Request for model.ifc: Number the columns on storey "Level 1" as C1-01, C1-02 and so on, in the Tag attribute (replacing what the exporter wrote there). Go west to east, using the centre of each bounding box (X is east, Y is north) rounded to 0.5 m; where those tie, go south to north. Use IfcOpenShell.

First a look at what the model holds.

```python
import ifcopenshell
import ifcopenshell.util.element
import ifcopenshell.util.placement

model = ifcopenshell.open("model.ifc")
print(model.schema)
storey = next(s for s in model.by_type("IfcBuildingStorey") if s.Name == "Level 1")
columns = [e for e in ifcopenshell.util.element.get_decomposition(storey) if e.is_a("IfcColumn")]
for e in sorted(columns, key=lambda e: e.id()):
    origin = ifcopenshell.util.placement.get_local_placement(e.ObjectPlacement)[:3, 3]
    print(e.id(), e.Tag, e.Name, origin.round(2) + 0.0, sep=" | ")
```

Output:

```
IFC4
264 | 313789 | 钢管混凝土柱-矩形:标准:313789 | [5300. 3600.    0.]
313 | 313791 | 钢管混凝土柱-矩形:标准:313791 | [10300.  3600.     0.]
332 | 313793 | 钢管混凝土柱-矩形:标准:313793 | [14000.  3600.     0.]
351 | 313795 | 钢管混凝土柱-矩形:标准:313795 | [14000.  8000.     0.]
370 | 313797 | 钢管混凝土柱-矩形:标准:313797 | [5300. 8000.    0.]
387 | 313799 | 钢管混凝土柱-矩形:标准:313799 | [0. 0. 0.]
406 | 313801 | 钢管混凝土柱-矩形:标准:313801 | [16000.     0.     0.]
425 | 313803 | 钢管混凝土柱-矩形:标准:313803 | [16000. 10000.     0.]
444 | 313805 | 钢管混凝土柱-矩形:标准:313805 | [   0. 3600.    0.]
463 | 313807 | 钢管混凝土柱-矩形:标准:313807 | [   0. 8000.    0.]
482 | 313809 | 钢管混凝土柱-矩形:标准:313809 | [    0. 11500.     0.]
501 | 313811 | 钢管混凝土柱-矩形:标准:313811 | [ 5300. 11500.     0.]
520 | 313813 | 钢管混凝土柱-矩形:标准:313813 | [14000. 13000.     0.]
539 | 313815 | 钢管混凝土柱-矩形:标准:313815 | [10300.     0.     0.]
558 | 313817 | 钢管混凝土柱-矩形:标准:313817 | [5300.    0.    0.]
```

```python
import ifcopenshell
import ifcopenshell.geom
import ifcopenshell.util.element
import ifcopenshell.util.shape

model = ifcopenshell.open("model.ifc")
settings = ifcopenshell.geom.settings()
settings.set("use-world-coords", True)


def centre(element):
    shape = ifcopenshell.geom.create_shape(settings, element)
    return ifcopenshell.util.shape.get_bbox_centroid(shape.geometry)


storey = next(s for s in model.by_type("IfcBuildingStorey") if s.Name == "Level 1")
columns = [e for e in ifcopenshell.util.element.get_decomposition(storey) if e.is_a("IfcColumn")]

# Insertion points can sit at a corner or the storey origin, so sort by the geometry (in metres).
centres = {e: centre(e) for e in columns}
columns.sort(key=lambda e: (round(centres[e][0] / 0.5), centres[e][1]))

for i, e in enumerate(columns, start=1):
    number = f"C1-{i:02d}"
    e.Tag = number
    print(e.id(), number)

model.write("model_updated.ifc")
```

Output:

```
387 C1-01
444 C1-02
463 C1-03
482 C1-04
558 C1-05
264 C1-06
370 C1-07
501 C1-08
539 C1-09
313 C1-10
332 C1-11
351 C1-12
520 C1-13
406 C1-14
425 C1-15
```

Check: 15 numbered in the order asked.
